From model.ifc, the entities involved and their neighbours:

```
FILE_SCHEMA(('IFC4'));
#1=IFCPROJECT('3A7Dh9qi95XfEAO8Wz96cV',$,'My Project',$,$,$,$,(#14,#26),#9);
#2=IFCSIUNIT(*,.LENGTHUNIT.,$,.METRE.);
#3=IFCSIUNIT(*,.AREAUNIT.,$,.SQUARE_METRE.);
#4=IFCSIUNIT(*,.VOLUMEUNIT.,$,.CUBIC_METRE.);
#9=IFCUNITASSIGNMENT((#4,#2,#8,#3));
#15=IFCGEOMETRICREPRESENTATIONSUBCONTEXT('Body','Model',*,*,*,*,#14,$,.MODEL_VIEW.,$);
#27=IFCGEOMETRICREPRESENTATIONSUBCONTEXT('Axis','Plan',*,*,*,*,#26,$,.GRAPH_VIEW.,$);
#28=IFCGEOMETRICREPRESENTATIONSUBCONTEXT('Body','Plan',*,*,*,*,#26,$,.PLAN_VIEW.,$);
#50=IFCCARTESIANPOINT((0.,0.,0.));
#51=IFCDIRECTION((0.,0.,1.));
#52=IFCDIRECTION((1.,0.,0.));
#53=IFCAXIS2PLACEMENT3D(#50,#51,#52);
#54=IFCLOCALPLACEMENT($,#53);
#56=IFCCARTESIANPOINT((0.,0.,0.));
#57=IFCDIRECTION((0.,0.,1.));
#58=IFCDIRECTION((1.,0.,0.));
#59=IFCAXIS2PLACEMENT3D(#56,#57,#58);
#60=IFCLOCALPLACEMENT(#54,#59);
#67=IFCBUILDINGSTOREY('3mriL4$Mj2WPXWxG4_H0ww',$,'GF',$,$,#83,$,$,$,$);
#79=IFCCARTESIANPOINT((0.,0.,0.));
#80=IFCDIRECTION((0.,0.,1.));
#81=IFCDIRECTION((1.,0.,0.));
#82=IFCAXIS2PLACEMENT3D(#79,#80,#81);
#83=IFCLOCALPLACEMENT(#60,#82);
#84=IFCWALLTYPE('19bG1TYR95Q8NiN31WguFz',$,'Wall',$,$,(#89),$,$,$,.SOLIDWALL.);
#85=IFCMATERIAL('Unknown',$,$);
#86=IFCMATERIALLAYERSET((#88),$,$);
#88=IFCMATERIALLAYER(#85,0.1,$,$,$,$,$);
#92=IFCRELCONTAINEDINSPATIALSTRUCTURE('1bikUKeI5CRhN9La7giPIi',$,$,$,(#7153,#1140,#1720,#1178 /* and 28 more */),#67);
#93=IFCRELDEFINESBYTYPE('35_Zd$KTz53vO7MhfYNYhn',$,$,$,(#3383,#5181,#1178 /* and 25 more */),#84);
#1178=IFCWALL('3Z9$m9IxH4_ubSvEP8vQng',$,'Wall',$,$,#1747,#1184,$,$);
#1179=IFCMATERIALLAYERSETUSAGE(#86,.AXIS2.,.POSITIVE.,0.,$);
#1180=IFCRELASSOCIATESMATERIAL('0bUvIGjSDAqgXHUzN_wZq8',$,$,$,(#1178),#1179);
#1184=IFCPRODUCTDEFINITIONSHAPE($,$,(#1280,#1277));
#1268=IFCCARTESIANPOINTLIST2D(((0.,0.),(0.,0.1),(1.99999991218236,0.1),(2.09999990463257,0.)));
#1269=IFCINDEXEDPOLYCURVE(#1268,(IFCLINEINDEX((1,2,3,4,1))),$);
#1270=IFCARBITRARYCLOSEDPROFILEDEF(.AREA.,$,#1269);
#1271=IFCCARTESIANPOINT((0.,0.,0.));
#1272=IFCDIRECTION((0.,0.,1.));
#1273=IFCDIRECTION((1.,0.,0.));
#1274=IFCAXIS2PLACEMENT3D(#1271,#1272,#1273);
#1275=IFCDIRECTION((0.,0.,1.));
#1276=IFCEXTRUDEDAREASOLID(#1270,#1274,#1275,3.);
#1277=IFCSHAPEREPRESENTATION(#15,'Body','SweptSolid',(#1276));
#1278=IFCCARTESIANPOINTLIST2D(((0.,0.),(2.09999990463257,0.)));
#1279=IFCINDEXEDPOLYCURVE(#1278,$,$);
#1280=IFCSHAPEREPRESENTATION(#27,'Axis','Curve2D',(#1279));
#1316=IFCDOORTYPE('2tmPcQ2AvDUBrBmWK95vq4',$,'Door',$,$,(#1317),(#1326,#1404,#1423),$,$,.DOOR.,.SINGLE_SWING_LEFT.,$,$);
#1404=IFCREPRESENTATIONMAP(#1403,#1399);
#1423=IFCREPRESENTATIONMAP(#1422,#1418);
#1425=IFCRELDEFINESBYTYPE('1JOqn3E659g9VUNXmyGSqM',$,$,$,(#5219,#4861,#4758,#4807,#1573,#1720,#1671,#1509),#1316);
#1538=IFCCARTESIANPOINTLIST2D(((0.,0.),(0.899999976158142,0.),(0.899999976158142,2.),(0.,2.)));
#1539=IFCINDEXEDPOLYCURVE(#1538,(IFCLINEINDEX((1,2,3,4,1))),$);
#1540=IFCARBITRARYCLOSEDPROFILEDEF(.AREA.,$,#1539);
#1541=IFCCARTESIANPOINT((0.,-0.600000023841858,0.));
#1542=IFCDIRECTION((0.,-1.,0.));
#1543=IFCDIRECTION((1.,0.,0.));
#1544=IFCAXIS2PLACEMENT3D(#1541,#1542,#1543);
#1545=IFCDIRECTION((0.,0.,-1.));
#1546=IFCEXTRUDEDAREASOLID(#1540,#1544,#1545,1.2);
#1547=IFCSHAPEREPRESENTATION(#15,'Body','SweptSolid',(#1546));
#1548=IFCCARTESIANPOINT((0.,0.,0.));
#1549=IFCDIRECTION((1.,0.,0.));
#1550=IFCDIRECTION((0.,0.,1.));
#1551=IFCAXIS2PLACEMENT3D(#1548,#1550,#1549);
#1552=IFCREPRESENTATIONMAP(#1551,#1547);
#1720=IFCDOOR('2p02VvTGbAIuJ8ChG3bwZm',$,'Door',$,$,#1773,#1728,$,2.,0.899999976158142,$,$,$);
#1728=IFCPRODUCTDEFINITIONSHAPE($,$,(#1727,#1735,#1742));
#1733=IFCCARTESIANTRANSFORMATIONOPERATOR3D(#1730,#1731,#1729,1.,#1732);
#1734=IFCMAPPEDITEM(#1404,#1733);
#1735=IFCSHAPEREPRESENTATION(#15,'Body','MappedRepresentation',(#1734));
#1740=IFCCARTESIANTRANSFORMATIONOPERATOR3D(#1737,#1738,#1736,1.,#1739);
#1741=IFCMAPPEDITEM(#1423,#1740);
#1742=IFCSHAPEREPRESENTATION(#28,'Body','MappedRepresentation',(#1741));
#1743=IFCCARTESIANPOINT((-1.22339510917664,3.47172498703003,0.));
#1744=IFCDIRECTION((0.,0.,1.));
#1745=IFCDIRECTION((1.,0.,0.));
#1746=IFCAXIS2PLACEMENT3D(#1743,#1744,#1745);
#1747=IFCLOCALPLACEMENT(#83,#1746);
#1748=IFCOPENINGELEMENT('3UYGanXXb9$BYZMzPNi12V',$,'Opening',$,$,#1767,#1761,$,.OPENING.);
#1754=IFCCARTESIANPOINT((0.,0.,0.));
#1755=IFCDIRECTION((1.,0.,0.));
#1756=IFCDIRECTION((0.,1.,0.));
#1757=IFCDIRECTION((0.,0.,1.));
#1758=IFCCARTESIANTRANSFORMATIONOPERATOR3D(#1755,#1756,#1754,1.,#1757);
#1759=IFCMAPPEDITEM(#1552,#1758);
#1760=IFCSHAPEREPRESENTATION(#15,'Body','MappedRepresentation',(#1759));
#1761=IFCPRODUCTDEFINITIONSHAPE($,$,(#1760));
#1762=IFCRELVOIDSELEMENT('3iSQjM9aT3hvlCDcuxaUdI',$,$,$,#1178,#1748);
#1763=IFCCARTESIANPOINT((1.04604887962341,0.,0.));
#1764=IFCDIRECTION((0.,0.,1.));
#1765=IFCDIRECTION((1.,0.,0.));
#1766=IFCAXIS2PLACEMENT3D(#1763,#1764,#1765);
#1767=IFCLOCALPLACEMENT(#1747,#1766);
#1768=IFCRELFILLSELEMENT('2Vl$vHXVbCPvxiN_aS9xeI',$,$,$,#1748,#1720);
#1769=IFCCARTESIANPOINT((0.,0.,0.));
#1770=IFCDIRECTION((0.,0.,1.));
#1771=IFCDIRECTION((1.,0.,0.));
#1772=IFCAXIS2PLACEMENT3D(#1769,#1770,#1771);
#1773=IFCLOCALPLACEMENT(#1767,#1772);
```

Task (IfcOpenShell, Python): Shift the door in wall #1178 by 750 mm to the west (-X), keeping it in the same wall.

```python
import ifcopenshell
import ifcopenshell.api.geometry
import ifcopenshell.util.placement

model = ifcopenshell.open("model.ifc")

door = model.by_guid("2p02VvTGbAIuJ8ChG3bwZm")
opening = door.FillsVoids[0].RelatingOpeningElement
wall = opening.VoidsElements[0].RelatingBuildingElement

wall_matrix = ifcopenshell.util.placement.get_local_placement(wall.ObjectPlacement)
shift = wall_matrix[:3, 0] * -0.75
before = ifcopenshell.util.placement.get_local_placement(door.ObjectPlacement)[:3, 3].copy()

# The door is placed relative to its opening, so it follows when the opening moves.
matrix = ifcopenshell.util.placement.get_local_placement(opening.ObjectPlacement)
matrix[:3, 3] += shift
ifcopenshell.api.geometry.edit_object_placement(
    model, product=opening, matrix=matrix, is_si=False, should_transform_children=True
)

after = ifcopenshell.util.placement.get_local_placement(door.ObjectPlacement)[:3, 3]
print("door moved by", (after - before).round(3) + 0.0)

model.write("model_v2.ifc")
```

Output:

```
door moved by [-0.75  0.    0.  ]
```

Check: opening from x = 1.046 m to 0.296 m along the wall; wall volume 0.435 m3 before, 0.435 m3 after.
